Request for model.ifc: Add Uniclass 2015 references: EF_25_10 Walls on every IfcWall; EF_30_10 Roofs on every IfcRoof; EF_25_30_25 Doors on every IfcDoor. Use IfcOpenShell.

First a look at what the model holds.

```python
import ifcopenshell

model = ifcopenshell.open("model.ifc")
print(model.schema)
print("classifications:", [c.Name for c in model.by_type("IfcClassification")])
for ifc_class in ("IfcDoor", "IfcRoof", "IfcStair", "IfcWall", "IfcWindow"):
    print(ifc_class, len(model.by_type(ifc_class)))
```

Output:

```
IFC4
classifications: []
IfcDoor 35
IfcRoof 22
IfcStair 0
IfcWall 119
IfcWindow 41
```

```python
import ifcopenshell
import ifcopenshell.api.classification

model = ifcopenshell.open("model.ifc")

system = ifcopenshell.api.classification.add_classification(model, classification="Uniclass 2015")

codes = {
    "IfcWall": ("EF_25_10", "Walls"),
    "IfcRoof": ("EF_30_10", "Roofs"),
    "IfcDoor": ("EF_25_30_25", "Doors"),
}
for ifc_class, (code, name) in codes.items():
    products = model.by_type(ifc_class)
    ifcopenshell.api.classification.add_reference(
        model, products=products, classification=system, identification=code, name=name
    )
    print(code, len(products))

model.write("model-out.ifc")
```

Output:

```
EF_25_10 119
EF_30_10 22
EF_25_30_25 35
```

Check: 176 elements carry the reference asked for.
